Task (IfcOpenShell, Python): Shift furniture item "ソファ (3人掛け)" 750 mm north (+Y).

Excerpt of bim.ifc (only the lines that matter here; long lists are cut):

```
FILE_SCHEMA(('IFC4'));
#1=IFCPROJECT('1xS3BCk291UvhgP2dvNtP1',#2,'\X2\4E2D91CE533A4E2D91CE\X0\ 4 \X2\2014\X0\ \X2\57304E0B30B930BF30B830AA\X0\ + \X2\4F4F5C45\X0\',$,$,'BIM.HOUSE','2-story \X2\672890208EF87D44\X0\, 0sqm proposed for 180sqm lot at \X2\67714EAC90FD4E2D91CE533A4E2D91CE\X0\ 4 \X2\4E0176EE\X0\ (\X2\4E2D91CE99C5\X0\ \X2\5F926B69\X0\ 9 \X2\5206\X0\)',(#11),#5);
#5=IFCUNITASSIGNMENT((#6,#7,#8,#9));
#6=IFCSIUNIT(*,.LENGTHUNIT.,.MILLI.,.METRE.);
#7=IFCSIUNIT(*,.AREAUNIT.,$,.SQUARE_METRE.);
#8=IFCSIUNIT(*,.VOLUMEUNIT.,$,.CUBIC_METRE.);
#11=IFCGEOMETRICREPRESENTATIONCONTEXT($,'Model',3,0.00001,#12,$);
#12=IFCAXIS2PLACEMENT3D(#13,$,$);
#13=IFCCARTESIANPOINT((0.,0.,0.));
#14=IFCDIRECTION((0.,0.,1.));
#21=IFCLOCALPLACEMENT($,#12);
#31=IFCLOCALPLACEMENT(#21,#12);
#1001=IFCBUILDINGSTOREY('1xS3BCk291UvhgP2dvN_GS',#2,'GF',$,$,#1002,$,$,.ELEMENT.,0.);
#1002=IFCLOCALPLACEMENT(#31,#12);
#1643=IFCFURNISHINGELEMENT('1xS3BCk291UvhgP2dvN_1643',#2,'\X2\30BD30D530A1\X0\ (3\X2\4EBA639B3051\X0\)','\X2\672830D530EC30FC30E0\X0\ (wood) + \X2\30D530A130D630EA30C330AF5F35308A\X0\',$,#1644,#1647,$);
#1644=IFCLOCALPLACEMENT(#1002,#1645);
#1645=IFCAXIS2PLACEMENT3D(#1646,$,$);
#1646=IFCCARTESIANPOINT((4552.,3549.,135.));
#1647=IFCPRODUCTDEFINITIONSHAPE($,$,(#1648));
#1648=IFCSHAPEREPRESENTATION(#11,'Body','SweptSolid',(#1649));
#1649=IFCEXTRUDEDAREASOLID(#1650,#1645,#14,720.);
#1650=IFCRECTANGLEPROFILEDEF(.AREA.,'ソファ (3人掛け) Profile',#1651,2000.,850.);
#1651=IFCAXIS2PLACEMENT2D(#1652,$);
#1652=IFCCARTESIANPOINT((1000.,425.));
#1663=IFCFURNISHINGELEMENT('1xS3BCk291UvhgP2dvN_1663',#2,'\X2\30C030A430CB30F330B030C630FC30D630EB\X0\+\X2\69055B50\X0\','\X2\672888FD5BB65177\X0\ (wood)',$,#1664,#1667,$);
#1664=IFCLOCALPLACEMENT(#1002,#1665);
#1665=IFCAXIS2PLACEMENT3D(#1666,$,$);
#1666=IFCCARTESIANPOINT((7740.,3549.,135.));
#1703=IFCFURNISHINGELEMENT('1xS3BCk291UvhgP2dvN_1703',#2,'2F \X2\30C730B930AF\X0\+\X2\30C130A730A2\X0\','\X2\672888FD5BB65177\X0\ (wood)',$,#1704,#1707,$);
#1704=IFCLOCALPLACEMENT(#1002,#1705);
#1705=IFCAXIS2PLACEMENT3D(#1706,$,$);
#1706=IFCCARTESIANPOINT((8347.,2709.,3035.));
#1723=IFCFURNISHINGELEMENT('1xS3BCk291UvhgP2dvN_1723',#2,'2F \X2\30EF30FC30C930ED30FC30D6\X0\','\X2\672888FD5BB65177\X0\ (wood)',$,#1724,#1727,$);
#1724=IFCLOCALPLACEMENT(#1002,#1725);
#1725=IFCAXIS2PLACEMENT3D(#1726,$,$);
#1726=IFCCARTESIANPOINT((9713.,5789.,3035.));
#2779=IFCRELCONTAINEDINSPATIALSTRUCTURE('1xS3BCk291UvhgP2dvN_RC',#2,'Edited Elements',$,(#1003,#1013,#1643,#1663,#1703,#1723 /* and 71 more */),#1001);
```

```python
import ifcopenshell
import ifcopenshell.api.geometry
import ifcopenshell.util.placement
import ifcopenshell.util.unit

model = ifcopenshell.open("bim.ifc")
unit_scale = ifcopenshell.util.unit.calculate_unit_scale(model)

item = model.by_id(1643)
matrix = ifcopenshell.util.placement.get_local_placement(item.ObjectPlacement)
matrix[1, 3] += 0.75 / unit_scale
ifcopenshell.api.geometry.edit_object_placement(model, product=item, matrix=matrix, is_si=False)

print(ifcopenshell.util.placement.get_local_placement(item.ObjectPlacement).round(3) + 0.0)

model.write("bim_updated.ifc")
```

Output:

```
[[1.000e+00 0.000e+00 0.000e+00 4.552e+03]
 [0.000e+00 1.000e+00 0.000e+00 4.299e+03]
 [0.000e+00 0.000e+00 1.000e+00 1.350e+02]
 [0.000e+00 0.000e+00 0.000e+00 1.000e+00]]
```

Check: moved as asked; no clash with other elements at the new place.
